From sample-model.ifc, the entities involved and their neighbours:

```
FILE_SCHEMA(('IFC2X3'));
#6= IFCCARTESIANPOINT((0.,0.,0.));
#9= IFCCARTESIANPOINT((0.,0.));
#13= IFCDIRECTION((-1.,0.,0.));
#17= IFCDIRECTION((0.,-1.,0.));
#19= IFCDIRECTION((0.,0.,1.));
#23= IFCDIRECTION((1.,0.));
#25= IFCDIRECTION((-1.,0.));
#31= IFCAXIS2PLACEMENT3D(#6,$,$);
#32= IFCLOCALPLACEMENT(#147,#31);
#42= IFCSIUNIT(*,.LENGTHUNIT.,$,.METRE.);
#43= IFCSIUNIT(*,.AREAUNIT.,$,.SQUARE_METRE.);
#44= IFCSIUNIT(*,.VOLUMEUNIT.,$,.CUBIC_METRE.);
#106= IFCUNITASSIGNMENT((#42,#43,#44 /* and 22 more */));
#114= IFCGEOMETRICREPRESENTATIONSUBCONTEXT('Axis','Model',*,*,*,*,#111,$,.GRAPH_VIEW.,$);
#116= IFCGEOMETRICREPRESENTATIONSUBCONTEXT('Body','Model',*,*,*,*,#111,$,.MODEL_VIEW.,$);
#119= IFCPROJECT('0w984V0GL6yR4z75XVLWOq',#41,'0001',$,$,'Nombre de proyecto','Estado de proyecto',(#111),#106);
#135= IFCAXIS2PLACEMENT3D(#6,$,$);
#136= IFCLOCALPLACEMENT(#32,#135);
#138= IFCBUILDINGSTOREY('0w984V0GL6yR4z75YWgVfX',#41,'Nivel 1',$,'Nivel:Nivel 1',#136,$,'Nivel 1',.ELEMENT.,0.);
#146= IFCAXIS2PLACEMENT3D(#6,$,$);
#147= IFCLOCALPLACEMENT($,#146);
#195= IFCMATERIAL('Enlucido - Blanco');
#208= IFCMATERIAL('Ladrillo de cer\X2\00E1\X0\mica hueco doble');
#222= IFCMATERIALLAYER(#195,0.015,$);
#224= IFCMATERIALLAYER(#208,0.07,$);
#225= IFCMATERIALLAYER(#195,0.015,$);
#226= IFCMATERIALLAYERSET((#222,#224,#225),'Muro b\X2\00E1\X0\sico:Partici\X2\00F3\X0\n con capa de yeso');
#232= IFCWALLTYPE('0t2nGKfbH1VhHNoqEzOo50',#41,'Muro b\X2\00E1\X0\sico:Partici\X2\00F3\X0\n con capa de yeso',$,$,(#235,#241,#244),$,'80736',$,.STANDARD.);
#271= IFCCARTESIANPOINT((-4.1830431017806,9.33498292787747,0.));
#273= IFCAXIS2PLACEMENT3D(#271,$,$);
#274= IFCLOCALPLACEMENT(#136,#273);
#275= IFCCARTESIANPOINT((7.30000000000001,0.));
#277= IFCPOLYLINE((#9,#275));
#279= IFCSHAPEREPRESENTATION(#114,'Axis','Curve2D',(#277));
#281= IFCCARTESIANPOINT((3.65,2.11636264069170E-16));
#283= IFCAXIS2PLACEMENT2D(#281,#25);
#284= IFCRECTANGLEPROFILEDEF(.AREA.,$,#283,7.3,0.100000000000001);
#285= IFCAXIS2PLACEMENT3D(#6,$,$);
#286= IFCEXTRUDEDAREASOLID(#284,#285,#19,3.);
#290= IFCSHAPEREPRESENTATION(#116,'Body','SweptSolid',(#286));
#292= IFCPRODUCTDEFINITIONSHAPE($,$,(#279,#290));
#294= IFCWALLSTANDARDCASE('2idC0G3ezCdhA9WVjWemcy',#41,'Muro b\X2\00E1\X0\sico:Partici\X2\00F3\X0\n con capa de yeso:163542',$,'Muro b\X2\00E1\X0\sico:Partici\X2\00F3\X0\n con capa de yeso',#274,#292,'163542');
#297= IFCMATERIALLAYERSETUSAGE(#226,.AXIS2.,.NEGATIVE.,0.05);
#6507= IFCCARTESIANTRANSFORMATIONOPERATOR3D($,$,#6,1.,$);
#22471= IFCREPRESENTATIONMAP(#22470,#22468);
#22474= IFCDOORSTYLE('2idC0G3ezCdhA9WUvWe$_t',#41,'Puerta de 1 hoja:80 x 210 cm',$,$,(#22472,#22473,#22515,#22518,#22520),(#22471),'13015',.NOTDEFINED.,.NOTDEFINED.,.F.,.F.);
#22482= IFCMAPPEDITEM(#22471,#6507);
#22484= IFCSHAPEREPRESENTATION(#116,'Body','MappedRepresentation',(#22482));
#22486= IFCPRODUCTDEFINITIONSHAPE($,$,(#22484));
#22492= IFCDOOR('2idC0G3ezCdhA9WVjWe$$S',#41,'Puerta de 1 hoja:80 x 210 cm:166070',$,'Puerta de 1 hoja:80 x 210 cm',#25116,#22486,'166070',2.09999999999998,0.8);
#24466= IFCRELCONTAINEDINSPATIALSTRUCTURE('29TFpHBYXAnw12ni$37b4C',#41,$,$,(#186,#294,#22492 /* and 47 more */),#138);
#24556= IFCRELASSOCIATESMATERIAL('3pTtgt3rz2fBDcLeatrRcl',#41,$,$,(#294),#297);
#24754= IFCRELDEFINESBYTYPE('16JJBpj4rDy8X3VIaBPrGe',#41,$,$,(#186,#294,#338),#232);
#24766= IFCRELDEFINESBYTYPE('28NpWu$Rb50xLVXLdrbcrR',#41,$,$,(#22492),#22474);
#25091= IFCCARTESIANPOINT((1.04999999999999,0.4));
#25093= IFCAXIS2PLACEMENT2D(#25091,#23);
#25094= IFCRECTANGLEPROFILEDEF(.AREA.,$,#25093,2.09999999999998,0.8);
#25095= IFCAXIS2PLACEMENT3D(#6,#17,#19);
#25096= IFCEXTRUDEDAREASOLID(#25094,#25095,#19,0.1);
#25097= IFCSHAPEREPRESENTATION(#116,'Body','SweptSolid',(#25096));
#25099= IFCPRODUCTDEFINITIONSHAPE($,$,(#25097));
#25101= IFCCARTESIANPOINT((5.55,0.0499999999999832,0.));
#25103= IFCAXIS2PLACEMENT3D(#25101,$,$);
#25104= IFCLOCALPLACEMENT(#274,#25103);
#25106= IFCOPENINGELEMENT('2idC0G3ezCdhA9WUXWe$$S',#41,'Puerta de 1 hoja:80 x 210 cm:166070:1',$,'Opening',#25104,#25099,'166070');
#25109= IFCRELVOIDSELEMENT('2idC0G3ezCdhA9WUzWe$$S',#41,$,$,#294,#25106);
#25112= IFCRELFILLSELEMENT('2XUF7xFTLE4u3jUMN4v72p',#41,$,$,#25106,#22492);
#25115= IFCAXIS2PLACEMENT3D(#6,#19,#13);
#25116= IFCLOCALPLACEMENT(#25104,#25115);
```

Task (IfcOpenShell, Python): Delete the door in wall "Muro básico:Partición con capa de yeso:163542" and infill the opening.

```python
import ifcopenshell
import ifcopenshell.api.feature
import ifcopenshell.api.root
import ifcopenshell.geom
import ifcopenshell.util.shape

model = ifcopenshell.open("sample-model.ifc")
settings = ifcopenshell.geom.settings()


def volume(element):
    """Net volume in cubic metres, openings subtracted."""
    shape = ifcopenshell.geom.create_shape(settings, element)
    return ifcopenshell.util.shape.get_volume(shape.geometry)


door = model.by_guid("2idC0G3ezCdhA9WVjWe$$S")
opening = door.FillsVoids[0].RelatingOpeningElement
wall = opening.VoidsElements[0].RelatingBuildingElement
before = volume(wall)

ifcopenshell.api.root.remove_product(model, product=door)
ifcopenshell.api.feature.remove_feature(model, feature=opening)

after = volume(wall)

print(f"wall volume {before:.3f} -> {after:.3f} m3")

model.write("sample-model_rev.ifc")
```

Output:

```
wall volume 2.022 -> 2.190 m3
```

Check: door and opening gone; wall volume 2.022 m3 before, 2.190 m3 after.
